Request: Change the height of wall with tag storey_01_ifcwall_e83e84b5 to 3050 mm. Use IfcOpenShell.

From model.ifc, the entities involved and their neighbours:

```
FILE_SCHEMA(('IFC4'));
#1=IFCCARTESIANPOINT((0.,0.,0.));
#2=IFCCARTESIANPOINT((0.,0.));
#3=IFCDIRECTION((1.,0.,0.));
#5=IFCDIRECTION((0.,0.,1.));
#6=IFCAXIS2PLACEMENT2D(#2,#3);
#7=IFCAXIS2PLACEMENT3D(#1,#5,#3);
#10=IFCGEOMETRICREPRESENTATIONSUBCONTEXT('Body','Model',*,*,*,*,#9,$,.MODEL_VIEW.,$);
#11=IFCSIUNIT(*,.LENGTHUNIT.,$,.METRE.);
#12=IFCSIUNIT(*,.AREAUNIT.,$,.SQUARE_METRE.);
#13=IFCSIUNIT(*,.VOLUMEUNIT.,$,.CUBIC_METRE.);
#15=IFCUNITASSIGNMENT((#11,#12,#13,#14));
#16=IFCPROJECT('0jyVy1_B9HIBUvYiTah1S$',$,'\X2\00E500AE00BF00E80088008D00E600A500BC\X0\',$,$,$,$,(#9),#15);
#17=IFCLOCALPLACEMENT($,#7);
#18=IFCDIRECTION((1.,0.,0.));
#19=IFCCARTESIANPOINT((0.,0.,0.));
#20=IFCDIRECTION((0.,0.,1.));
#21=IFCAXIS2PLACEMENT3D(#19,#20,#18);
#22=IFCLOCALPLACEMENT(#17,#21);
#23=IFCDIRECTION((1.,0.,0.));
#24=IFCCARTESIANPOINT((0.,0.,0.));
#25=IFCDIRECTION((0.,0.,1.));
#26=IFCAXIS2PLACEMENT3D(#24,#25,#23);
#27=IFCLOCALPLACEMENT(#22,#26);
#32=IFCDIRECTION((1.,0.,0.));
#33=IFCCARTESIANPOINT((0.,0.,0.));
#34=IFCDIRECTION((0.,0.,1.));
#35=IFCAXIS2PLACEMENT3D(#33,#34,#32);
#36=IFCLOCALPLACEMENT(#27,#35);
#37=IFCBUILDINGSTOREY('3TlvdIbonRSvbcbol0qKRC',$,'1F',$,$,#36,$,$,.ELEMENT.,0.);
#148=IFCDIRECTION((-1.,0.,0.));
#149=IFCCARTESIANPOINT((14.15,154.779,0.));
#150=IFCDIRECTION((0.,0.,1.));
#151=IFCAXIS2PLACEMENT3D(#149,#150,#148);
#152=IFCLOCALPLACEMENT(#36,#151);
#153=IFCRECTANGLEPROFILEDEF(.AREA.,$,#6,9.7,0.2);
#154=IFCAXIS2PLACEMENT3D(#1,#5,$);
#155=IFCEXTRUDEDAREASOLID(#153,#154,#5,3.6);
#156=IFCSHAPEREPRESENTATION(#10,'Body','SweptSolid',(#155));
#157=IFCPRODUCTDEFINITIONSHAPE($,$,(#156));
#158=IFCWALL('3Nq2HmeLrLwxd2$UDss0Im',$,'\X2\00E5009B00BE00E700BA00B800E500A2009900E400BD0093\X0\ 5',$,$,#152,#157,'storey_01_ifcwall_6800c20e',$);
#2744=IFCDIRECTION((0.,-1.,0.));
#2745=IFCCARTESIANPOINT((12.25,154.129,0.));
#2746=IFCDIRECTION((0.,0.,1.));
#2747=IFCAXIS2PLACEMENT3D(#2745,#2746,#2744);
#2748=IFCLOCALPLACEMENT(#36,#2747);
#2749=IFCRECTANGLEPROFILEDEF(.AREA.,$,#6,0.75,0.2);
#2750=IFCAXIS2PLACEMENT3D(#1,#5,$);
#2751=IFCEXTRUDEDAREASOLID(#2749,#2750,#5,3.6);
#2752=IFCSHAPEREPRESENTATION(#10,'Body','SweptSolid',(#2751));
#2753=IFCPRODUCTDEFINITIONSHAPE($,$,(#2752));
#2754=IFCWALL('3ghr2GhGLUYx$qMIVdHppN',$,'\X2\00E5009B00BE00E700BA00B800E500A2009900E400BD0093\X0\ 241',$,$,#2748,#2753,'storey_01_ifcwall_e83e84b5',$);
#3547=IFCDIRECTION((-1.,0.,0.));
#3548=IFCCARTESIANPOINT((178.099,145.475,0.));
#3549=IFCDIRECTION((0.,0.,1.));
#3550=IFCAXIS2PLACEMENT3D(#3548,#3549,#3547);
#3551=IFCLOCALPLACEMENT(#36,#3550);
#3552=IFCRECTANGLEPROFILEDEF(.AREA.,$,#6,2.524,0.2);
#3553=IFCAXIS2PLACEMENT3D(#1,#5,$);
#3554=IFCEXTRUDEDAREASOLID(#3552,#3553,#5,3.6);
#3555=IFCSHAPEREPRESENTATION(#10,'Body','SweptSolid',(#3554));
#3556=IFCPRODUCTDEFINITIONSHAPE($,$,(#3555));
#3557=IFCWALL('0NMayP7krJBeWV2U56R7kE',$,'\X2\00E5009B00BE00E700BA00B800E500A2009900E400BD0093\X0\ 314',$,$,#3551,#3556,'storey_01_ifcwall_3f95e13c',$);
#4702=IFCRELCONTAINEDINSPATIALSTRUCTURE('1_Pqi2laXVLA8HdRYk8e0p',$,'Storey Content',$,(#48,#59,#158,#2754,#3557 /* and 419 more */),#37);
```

```python
import ifcopenshell
import ifcopenshell.geom
import ifcopenshell.util.representation
import ifcopenshell.util.shape

model = ifcopenshell.open("model.ifc")
settings = ifcopenshell.geom.settings()


def volume(element):
    """Net volume in cubic metres, openings subtracted."""
    shape = ifcopenshell.geom.create_shape(settings, element)
    return ifcopenshell.util.shape.get_volume(shape.geometry)


wall = model.by_id(2754)
before = volume(wall)

body = ifcopenshell.util.representation.get_representation(wall, "Model", "Body")
solid = body.Items[0]
old_height = solid.Depth
solid.Depth = 3.05
after = volume(wall)

print(f"height {old_height:g} -> {solid.Depth:g}, volume {before:.3f} -> {after:.3f} m3")

model.write("model_rev.ifc")
```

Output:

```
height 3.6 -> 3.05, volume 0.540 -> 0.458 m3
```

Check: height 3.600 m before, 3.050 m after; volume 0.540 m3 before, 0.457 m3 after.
